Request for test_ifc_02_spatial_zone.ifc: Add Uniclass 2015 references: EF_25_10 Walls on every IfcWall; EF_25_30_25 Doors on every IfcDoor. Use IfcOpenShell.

First a look at what the model holds.

```python
import ifcopenshell

model = ifcopenshell.open("test_ifc_02_spatial_zone.ifc")
print(model.schema)
print("classifications:", [c.Name for c in model.by_type("IfcClassification")])
for ifc_class in ("IfcDoor", "IfcRoof", "IfcStair", "IfcWall", "IfcWindow"):
    print(ifc_class, len(model.by_type(ifc_class)))
```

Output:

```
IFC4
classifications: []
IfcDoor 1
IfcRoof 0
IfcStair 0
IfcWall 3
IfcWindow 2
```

```python
import ifcopenshell
import ifcopenshell.api.classification

model = ifcopenshell.open("test_ifc_02_spatial_zone.ifc")

system = ifcopenshell.api.classification.add_classification(model, classification="Uniclass 2015")

codes = {
    "IfcWall": ("EF_25_10", "Walls"),
    "IfcDoor": ("EF_25_30_25", "Doors"),
}
for ifc_class, (code, name) in codes.items():
    products = model.by_type(ifc_class)
    ifcopenshell.api.classification.add_reference(
        model, products=products, classification=system, identification=code, name=name
    )
    print(code, len(products))

model.write("test_ifc_02_spatial_zone_rev.ifc")
```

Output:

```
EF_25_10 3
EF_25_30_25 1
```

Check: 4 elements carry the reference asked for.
